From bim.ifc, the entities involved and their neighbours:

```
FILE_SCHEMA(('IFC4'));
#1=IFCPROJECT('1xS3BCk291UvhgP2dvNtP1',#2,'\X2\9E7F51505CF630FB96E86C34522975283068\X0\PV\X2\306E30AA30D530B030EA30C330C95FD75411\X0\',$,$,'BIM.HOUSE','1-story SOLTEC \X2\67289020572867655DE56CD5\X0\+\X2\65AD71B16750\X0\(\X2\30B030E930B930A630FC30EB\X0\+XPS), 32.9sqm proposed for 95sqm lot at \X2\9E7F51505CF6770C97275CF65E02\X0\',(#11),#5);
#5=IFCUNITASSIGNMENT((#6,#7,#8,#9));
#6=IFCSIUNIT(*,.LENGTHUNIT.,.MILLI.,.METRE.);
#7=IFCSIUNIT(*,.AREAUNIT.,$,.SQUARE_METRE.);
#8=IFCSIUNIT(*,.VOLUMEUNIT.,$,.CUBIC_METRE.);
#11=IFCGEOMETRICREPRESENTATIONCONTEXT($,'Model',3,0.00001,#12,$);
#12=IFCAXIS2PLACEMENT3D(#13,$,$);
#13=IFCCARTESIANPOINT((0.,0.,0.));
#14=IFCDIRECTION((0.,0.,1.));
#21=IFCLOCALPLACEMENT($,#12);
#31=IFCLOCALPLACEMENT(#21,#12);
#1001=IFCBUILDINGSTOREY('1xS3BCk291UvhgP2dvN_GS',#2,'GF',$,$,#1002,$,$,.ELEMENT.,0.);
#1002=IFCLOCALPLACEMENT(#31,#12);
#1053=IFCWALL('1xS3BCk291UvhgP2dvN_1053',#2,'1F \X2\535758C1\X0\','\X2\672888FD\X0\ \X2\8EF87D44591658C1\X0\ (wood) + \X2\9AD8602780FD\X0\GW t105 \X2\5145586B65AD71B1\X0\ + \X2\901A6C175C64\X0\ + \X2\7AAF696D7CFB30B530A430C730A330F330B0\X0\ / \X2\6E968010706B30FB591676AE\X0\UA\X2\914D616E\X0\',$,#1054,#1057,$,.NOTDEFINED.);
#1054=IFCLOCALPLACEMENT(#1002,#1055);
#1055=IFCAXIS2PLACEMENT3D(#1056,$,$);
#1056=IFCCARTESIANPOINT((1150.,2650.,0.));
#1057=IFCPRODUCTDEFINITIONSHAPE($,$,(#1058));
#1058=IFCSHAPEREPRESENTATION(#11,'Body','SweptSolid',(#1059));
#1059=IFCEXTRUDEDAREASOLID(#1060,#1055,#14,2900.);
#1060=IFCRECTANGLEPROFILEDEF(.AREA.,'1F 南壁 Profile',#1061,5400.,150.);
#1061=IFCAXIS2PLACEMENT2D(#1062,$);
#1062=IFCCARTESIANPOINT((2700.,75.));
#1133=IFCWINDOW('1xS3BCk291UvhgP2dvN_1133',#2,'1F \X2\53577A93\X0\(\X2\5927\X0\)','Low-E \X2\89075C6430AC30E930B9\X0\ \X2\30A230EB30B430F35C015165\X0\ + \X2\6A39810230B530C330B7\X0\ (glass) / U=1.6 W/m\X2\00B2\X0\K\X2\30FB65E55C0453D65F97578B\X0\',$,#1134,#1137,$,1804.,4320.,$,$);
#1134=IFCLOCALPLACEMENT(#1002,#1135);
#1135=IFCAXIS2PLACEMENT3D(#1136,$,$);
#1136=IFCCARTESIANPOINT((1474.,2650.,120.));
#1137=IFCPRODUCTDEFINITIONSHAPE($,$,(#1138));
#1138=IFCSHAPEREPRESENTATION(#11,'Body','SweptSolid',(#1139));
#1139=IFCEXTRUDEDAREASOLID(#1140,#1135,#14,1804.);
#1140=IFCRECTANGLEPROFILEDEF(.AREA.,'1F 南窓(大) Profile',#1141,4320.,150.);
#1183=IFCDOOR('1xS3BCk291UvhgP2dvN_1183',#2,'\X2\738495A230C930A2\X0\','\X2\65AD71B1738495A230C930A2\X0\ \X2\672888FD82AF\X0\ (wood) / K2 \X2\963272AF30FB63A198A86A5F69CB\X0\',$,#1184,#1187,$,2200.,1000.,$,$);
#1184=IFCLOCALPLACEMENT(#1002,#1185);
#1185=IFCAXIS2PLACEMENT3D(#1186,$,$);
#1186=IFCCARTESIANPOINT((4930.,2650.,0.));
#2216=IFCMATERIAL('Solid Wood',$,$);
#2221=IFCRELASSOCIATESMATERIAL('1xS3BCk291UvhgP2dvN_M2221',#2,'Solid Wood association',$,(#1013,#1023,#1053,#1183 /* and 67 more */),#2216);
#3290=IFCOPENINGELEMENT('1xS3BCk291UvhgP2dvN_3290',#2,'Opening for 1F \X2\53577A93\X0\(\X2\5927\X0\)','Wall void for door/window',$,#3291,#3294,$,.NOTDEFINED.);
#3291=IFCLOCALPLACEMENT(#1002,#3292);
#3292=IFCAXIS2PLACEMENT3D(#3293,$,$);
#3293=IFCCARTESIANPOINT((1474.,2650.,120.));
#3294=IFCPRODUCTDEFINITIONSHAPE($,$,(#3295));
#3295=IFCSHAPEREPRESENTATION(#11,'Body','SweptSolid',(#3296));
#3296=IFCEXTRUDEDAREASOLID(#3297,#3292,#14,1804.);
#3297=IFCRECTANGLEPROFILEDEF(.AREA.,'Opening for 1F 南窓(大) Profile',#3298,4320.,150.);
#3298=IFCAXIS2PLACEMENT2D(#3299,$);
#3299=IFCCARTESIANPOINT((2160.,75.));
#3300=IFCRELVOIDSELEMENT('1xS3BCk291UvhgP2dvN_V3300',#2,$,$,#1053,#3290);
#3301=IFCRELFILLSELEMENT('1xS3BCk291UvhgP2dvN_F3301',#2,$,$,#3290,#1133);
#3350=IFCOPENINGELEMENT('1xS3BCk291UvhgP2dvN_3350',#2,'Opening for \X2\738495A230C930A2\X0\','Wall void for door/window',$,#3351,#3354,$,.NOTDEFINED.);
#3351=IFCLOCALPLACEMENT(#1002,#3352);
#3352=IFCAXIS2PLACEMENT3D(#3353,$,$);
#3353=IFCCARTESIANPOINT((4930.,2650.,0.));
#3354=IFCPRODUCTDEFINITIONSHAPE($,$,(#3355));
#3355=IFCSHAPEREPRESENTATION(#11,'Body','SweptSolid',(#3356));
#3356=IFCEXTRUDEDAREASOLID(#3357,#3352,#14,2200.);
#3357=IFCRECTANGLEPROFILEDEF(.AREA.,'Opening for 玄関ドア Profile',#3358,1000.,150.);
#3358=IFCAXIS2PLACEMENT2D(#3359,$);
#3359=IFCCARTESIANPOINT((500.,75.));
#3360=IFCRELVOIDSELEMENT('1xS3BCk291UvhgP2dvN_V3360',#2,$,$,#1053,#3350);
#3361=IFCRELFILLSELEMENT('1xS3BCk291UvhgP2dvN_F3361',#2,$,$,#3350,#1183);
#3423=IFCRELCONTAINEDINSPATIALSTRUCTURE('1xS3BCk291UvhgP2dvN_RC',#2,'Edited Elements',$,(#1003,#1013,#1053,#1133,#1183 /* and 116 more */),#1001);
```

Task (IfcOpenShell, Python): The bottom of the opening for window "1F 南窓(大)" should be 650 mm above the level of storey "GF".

```python
import numpy as np
import ifcopenshell
import ifcopenshell.api.geometry
import ifcopenshell.geom
import ifcopenshell.util.element
import ifcopenshell.util.placement
import ifcopenshell.util.shape
import ifcopenshell.util.unit

model = ifcopenshell.open("bim.ifc")
unit_scale = ifcopenshell.util.unit.calculate_unit_scale(model)

window = model.by_guid("1xS3BCk291UvhgP2dvN_1133")
opening = window.FillsVoids[0].RelatingOpeningElement
storey = ifcopenshell.util.element.get_container(window, ifc_class="IfcBuildingStorey")
level = ifcopenshell.util.placement.get_local_placement(storey.ObjectPlacement)[2, 3]

# The opening's origin need not be at the sill, so measure its lowest point.
shape = ifcopenshell.geom.create_shape(ifcopenshell.geom.settings(), opening)
bottom = ifcopenshell.util.shape.get_shape_bottom_elevation(shape, shape.geometry) / unit_scale
dz = level + 0.65 / unit_scale - bottom

shift = np.array([0.0, 0.0, dz])
# The window is not placed relative to its opening, so move both.
for product in (opening, window):
    matrix = ifcopenshell.util.placement.get_local_placement(product.ObjectPlacement)
    matrix[:3, 3] += shift
    ifcopenshell.api.geometry.edit_object_placement(model, product=product, matrix=matrix, is_si=False)

print(f"moved by {dz * unit_scale:+.3f} m")

model.write("bim-out.ifc")
```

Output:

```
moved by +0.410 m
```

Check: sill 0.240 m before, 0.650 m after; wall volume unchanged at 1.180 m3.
